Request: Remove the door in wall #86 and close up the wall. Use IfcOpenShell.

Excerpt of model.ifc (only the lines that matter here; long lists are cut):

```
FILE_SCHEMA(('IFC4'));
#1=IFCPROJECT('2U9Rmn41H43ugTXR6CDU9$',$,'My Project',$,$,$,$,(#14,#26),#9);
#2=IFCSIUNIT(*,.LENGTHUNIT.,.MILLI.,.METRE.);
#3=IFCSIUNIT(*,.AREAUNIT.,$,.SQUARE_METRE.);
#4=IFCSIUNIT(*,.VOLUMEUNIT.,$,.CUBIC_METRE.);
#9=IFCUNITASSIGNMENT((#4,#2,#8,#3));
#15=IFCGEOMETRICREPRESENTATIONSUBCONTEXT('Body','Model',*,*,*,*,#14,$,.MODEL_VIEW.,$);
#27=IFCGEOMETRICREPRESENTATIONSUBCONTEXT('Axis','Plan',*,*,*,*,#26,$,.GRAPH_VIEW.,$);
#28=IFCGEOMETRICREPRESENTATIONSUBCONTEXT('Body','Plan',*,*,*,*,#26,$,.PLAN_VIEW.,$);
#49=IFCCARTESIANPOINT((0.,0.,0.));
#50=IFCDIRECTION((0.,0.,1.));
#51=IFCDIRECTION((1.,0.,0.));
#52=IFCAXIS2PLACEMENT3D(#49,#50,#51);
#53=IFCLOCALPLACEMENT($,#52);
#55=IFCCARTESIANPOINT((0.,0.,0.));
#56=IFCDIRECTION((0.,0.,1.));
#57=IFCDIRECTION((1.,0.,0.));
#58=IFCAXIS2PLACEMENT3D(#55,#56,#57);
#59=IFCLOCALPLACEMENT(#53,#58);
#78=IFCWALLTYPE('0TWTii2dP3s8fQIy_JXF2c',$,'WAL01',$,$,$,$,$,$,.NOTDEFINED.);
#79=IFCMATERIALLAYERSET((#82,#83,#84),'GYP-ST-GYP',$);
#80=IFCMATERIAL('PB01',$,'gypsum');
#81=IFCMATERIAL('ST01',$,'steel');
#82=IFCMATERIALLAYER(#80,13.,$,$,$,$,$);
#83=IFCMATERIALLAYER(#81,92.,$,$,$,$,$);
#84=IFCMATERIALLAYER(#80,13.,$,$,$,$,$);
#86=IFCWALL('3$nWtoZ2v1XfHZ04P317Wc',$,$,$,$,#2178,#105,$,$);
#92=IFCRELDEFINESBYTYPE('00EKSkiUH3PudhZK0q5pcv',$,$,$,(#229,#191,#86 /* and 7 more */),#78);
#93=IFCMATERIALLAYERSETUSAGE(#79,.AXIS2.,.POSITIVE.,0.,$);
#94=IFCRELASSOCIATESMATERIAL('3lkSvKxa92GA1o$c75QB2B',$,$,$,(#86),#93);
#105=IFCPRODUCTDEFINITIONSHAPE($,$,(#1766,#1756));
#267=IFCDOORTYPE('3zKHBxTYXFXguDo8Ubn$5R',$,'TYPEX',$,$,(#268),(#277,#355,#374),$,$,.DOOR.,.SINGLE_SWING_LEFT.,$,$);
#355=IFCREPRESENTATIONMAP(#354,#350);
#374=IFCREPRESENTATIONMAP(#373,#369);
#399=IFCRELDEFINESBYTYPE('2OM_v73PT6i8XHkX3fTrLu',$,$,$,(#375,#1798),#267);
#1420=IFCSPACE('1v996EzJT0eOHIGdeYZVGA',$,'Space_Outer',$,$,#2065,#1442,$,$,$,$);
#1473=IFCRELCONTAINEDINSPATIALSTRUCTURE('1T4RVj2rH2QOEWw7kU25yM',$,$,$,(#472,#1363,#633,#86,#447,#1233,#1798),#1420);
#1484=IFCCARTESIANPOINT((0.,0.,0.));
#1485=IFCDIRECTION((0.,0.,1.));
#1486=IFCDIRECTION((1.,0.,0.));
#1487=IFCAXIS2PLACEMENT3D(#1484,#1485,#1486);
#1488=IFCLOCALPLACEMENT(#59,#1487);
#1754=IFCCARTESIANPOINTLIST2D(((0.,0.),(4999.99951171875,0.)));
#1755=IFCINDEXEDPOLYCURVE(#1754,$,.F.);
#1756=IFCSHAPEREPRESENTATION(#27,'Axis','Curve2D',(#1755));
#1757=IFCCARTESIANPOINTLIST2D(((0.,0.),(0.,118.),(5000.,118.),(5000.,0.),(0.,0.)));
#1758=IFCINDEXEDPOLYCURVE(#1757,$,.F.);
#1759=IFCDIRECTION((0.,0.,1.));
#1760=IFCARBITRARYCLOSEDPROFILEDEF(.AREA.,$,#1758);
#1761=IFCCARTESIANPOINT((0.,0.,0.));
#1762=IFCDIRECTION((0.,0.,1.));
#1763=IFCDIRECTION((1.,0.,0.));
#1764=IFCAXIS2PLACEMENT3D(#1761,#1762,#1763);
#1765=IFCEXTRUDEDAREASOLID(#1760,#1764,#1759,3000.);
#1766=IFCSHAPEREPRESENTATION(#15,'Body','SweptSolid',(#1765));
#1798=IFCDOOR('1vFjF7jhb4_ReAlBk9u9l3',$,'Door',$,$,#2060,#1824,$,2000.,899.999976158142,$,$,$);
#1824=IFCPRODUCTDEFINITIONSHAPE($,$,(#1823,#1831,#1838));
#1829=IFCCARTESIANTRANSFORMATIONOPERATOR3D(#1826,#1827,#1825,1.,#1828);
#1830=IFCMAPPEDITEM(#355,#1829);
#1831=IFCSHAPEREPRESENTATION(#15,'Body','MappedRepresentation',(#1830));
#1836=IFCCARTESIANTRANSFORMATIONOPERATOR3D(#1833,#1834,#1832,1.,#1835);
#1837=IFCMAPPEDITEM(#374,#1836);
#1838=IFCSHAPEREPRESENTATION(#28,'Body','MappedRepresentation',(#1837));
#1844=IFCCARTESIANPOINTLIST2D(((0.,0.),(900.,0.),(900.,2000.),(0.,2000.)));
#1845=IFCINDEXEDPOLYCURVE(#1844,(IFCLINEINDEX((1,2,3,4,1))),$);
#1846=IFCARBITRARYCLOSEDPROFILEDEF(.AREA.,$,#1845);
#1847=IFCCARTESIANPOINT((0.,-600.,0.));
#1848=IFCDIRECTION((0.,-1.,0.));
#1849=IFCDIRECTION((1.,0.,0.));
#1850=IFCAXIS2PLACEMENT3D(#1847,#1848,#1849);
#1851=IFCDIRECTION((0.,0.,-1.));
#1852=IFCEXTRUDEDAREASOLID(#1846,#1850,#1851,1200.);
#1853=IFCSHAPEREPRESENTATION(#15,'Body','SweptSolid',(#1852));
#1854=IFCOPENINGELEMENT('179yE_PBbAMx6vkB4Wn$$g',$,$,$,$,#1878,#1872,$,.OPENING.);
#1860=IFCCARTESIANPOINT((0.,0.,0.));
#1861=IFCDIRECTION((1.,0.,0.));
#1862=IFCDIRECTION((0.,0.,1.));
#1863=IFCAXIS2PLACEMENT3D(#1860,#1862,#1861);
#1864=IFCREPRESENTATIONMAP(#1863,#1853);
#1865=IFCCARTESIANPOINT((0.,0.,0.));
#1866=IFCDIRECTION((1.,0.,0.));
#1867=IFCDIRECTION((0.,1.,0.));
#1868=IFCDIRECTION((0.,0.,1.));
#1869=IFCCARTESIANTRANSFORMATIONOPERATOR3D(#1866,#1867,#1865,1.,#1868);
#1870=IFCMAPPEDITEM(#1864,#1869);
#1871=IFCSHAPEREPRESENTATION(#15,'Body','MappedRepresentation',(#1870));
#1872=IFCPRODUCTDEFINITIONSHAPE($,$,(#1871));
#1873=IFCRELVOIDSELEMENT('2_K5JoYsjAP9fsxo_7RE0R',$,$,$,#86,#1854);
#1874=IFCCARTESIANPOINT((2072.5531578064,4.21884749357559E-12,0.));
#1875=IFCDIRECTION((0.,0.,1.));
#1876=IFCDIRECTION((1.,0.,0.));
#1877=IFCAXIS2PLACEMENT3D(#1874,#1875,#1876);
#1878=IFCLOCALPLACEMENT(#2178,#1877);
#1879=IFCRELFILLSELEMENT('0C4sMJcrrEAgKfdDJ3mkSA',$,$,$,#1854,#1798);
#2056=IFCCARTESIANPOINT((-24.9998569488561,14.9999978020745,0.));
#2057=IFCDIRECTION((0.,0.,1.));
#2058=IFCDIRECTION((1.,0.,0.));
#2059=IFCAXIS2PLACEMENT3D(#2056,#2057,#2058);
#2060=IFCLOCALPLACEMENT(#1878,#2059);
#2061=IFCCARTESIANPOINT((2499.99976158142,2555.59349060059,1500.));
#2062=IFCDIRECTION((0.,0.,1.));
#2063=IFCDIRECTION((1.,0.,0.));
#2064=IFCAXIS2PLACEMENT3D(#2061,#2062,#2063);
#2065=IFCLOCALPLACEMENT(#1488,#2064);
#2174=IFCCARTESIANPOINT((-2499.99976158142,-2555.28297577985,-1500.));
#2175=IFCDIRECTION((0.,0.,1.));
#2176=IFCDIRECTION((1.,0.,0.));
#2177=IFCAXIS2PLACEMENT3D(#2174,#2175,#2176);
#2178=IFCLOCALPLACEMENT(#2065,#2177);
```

```python
import ifcopenshell
import ifcopenshell.api.feature
import ifcopenshell.api.root
import ifcopenshell.geom
import ifcopenshell.util.shape

model = ifcopenshell.open("model.ifc")
settings = ifcopenshell.geom.settings()


def volume(element):
    """Net volume in cubic metres, openings subtracted."""
    shape = ifcopenshell.geom.create_shape(settings, element)
    return ifcopenshell.util.shape.get_volume(shape.geometry)


door = model.by_guid("1vFjF7jhb4_ReAlBk9u9l3")
opening = door.FillsVoids[0].RelatingOpeningElement
wall = opening.VoidsElements[0].RelatingBuildingElement
before = volume(wall)

ifcopenshell.api.root.remove_product(model, product=door)
ifcopenshell.api.feature.remove_feature(model, feature=opening)

after = volume(wall)

print(f"wall volume {before:.3f} -> {after:.3f} m3")

model.write("model_edited.ifc")
```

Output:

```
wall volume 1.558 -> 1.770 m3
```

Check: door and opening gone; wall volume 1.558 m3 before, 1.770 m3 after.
